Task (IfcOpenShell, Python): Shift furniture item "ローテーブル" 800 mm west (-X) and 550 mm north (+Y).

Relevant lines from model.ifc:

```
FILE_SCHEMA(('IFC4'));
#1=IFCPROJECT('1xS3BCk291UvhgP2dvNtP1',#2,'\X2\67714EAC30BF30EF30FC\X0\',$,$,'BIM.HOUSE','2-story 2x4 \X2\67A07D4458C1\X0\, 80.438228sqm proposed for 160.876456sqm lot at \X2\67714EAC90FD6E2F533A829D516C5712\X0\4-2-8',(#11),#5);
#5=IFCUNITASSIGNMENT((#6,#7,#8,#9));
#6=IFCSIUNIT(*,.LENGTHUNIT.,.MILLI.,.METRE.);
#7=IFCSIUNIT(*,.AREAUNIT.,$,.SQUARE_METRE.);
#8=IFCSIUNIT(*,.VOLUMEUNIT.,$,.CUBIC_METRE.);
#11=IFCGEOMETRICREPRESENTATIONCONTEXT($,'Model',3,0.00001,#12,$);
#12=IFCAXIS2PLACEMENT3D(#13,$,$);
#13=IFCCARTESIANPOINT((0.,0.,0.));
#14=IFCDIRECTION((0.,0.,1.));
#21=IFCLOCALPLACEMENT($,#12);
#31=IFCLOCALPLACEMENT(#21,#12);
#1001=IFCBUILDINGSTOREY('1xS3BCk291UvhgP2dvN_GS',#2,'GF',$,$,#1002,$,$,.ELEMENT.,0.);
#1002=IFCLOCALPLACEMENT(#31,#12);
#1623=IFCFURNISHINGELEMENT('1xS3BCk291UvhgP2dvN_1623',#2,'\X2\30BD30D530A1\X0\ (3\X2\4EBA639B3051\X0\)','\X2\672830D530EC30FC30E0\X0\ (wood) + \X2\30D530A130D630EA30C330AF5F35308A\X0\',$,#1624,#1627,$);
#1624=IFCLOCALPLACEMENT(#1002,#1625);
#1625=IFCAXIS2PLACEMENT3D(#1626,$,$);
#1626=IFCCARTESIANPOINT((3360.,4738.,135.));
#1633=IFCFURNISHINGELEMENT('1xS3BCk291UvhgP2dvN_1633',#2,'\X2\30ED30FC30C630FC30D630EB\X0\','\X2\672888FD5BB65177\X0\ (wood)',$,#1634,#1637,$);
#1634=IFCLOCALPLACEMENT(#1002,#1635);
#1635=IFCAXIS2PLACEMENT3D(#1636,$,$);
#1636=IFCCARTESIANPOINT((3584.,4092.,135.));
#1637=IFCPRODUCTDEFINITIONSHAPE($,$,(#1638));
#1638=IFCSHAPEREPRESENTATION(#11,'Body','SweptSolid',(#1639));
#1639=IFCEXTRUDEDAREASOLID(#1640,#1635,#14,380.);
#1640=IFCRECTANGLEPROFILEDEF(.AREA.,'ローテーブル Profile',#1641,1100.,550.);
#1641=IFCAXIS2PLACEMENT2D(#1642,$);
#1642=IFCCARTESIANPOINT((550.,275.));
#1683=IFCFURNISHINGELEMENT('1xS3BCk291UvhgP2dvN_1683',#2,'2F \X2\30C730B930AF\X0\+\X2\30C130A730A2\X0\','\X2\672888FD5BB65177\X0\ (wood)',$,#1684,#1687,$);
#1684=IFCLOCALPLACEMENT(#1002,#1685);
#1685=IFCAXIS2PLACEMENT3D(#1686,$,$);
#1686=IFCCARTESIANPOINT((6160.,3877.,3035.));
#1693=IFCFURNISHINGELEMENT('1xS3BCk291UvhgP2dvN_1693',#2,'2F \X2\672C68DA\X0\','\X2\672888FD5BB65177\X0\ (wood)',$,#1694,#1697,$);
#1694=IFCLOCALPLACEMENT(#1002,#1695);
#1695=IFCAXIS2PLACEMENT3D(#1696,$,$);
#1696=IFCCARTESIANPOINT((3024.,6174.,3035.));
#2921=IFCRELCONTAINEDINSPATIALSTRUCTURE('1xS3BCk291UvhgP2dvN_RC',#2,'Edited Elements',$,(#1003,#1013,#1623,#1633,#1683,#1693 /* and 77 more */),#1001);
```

```python
import ifcopenshell
import ifcopenshell.api.geometry
import ifcopenshell.util.placement

model = ifcopenshell.open("model.ifc")

item = model.by_id(1633)
matrix = ifcopenshell.util.placement.get_local_placement(item.ObjectPlacement)
matrix[0, 3] -= 800.0
matrix[1, 3] += 550.0
ifcopenshell.api.geometry.edit_object_placement(model, product=item, matrix=matrix, is_si=False)

print(ifcopenshell.util.placement.get_local_placement(item.ObjectPlacement).round(3) + 0.0)

model.write("model-out.ifc")
```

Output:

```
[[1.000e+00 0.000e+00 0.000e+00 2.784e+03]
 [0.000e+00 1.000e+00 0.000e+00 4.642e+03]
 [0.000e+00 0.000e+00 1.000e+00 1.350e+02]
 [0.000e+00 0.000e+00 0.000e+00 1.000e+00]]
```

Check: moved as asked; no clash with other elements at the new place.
